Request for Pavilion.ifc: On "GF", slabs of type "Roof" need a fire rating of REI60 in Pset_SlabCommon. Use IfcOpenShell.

First a look at what the model holds.

```python
import ifcopenshell
import ifcopenshell.util.element

model = ifcopenshell.open("Pavilion.ifc")
print(model.schema)
storey = next(s for s in model.by_type("IfcBuildingStorey") if s.Name == "GF")
slabs = [e for e in ifcopenshell.util.element.get_decomposition(storey) if e.is_a("IfcSlab")]
seen = {}
for e in slabs:
    element_type = ifcopenshell.util.element.get_type(e)
    key = (element_type.Name if element_type != e and element_type else None, ifcopenshell.util.element.get_pset(e, "Pset_SlabCommon", "FireRating"))
    seen[key] = seen.get(key, 0) + 1
for (name, value), count in sorted(seen.items(), key=str):
    print(count, "x", name, "|", value)
```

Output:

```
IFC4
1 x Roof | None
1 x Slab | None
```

```python
import ifcopenshell
import ifcopenshell.api.pset
import ifcopenshell.util.element

model = ifcopenshell.open("Pavilion.ifc")

storey = next(s for s in model.by_type("IfcBuildingStorey") if s.Name == "GF")
slabs = [e for e in ifcopenshell.util.element.get_decomposition(storey) if e.is_a("IfcSlab")]

count = 0
for e in slabs:
    element_type = ifcopenshell.util.element.get_type(e)
    if element_type in (None, e) or element_type.Name != "Roof":
        continue
    # add_pset returns the element's existing set when there is one.
    pset = ifcopenshell.api.pset.add_pset(model, product=e, name="Pset_SlabCommon")
    ifcopenshell.api.pset.edit_pset(model, pset=pset, properties={"FireRating": "REI60"})
    count += 1

print(count, "slabs updated")

model.write("Pavilion_updated.ifc")
```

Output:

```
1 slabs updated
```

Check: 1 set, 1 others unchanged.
